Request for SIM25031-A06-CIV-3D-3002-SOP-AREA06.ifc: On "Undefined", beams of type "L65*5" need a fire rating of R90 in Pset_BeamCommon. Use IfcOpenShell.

First a look at what the model holds.

```python
import ifcopenshell
import ifcopenshell.util.element

model = ifcopenshell.open("SIM25031-A06-CIV-3D-3002-SOP-AREA06.ifc")
print(model.schema)
storey = next(s for s in model.by_type("IfcBuildingStorey") if s.Name == "Undefined")
beams = [e for e in ifcopenshell.util.element.get_decomposition(storey) if e.is_a("IfcBeam")]
seen = {}
for e in beams:
    element_type = ifcopenshell.util.element.get_type(e)
    key = (element_type.Name if element_type != e and element_type else None, ifcopenshell.util.element.get_pset(e, "Pset_BeamCommon", "FireRating"))
    seen[key] = seen.get(key, 0) + 1
for (name, value), count in sorted(seen.items(), key=str):
    print(count, "x", name, "|", value)
```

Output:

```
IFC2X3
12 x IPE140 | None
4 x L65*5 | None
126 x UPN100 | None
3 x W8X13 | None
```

```python
import ifcopenshell
import ifcopenshell.api.pset
import ifcopenshell.util.element

model = ifcopenshell.open("SIM25031-A06-CIV-3D-3002-SOP-AREA06.ifc")

storey = next(s for s in model.by_type("IfcBuildingStorey") if s.Name == "Undefined")
beams = [e for e in ifcopenshell.util.element.get_decomposition(storey) if e.is_a("IfcBeam")]

count = 0
for e in beams:
    element_type = ifcopenshell.util.element.get_type(e)
    if element_type in (None, e) or element_type.Name != "L65*5":
        continue
    found = ifcopenshell.util.element.get_pset(e, "Pset_BeamCommon", should_inherit=False)
    if found:
        pset = model.by_id(found["id"])
        if len(ifcopenshell.util.element.get_elements_by_pset(pset)) > 1:
            pset = ifcopenshell.api.pset.unshare_pset(model, products=[e], pset=pset)[0]
    else:
        pset = ifcopenshell.api.pset.add_pset(model, product=e, name="Pset_BeamCommon")
    ifcopenshell.api.pset.edit_pset(model, pset=pset, properties={"FireRating": "R90"})
    count += 1

print(count, "beams updated")

model.write("SIM25031-A06-CIV-3D-3002-SOP-AREA06_v2.ifc")
```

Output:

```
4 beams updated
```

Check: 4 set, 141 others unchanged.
